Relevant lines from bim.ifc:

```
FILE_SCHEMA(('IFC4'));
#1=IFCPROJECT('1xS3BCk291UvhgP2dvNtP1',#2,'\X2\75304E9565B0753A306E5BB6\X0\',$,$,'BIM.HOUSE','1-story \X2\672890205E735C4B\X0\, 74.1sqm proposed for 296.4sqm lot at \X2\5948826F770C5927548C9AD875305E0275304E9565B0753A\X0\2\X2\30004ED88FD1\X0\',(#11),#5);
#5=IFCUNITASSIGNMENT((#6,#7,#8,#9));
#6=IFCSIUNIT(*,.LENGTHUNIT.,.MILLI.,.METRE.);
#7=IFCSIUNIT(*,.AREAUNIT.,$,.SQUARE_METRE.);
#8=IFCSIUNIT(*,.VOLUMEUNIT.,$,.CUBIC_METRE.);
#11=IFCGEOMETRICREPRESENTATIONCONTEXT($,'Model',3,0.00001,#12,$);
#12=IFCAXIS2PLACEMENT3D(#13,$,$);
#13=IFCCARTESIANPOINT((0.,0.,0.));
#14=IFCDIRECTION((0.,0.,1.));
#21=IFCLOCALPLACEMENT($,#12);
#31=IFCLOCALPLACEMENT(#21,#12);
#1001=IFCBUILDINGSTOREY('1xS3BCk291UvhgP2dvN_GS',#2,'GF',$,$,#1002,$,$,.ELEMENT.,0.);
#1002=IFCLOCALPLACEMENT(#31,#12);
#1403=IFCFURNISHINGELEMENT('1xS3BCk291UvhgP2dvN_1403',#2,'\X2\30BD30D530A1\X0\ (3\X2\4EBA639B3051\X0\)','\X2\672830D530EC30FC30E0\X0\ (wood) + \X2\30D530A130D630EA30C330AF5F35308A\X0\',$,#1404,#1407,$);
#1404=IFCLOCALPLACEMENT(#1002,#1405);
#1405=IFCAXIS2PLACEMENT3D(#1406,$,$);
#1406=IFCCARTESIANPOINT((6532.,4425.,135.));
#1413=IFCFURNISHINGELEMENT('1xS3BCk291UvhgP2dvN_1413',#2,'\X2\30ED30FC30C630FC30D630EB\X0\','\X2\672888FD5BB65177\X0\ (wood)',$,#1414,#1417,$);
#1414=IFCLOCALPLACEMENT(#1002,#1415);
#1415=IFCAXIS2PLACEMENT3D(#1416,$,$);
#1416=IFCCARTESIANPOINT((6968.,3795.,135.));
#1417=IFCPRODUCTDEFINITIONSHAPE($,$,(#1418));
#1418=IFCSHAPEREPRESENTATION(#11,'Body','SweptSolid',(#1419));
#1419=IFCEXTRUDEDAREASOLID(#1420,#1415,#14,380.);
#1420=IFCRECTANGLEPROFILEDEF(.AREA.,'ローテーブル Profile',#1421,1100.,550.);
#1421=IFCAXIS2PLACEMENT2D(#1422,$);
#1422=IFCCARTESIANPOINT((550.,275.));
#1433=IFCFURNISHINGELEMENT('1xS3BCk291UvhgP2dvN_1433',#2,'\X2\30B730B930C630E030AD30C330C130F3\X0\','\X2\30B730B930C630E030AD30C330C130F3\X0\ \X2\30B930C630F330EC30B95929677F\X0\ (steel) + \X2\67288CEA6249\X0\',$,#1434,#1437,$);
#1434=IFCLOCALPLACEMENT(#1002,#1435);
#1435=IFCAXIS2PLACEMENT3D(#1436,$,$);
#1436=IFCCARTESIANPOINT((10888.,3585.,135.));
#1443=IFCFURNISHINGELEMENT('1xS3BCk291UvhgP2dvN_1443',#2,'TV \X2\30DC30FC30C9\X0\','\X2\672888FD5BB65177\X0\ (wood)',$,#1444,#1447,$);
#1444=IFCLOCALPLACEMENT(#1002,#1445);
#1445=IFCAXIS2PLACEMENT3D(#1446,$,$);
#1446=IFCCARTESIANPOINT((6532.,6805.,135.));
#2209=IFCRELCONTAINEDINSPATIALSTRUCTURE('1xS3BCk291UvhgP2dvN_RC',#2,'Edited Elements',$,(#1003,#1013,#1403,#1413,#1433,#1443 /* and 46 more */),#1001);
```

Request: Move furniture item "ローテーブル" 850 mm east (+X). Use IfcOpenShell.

```python
import ifcopenshell
import ifcopenshell.api.geometry
import ifcopenshell.util.placement

model = ifcopenshell.open("bim.ifc")

item = model.by_guid("1xS3BCk291UvhgP2dvN_1413")
matrix = ifcopenshell.util.placement.get_local_placement(item.ObjectPlacement)
matrix[0, 3] += 850.0
ifcopenshell.api.geometry.edit_object_placement(model, product=item, matrix=matrix, is_si=False)

print(ifcopenshell.util.placement.get_local_placement(item.ObjectPlacement).round(3) + 0.0)

model.write("bim_v2.ifc")
```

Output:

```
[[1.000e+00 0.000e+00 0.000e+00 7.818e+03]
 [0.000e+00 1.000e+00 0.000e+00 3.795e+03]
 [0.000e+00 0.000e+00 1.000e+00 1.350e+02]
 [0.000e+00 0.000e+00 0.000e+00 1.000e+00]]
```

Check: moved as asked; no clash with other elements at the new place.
